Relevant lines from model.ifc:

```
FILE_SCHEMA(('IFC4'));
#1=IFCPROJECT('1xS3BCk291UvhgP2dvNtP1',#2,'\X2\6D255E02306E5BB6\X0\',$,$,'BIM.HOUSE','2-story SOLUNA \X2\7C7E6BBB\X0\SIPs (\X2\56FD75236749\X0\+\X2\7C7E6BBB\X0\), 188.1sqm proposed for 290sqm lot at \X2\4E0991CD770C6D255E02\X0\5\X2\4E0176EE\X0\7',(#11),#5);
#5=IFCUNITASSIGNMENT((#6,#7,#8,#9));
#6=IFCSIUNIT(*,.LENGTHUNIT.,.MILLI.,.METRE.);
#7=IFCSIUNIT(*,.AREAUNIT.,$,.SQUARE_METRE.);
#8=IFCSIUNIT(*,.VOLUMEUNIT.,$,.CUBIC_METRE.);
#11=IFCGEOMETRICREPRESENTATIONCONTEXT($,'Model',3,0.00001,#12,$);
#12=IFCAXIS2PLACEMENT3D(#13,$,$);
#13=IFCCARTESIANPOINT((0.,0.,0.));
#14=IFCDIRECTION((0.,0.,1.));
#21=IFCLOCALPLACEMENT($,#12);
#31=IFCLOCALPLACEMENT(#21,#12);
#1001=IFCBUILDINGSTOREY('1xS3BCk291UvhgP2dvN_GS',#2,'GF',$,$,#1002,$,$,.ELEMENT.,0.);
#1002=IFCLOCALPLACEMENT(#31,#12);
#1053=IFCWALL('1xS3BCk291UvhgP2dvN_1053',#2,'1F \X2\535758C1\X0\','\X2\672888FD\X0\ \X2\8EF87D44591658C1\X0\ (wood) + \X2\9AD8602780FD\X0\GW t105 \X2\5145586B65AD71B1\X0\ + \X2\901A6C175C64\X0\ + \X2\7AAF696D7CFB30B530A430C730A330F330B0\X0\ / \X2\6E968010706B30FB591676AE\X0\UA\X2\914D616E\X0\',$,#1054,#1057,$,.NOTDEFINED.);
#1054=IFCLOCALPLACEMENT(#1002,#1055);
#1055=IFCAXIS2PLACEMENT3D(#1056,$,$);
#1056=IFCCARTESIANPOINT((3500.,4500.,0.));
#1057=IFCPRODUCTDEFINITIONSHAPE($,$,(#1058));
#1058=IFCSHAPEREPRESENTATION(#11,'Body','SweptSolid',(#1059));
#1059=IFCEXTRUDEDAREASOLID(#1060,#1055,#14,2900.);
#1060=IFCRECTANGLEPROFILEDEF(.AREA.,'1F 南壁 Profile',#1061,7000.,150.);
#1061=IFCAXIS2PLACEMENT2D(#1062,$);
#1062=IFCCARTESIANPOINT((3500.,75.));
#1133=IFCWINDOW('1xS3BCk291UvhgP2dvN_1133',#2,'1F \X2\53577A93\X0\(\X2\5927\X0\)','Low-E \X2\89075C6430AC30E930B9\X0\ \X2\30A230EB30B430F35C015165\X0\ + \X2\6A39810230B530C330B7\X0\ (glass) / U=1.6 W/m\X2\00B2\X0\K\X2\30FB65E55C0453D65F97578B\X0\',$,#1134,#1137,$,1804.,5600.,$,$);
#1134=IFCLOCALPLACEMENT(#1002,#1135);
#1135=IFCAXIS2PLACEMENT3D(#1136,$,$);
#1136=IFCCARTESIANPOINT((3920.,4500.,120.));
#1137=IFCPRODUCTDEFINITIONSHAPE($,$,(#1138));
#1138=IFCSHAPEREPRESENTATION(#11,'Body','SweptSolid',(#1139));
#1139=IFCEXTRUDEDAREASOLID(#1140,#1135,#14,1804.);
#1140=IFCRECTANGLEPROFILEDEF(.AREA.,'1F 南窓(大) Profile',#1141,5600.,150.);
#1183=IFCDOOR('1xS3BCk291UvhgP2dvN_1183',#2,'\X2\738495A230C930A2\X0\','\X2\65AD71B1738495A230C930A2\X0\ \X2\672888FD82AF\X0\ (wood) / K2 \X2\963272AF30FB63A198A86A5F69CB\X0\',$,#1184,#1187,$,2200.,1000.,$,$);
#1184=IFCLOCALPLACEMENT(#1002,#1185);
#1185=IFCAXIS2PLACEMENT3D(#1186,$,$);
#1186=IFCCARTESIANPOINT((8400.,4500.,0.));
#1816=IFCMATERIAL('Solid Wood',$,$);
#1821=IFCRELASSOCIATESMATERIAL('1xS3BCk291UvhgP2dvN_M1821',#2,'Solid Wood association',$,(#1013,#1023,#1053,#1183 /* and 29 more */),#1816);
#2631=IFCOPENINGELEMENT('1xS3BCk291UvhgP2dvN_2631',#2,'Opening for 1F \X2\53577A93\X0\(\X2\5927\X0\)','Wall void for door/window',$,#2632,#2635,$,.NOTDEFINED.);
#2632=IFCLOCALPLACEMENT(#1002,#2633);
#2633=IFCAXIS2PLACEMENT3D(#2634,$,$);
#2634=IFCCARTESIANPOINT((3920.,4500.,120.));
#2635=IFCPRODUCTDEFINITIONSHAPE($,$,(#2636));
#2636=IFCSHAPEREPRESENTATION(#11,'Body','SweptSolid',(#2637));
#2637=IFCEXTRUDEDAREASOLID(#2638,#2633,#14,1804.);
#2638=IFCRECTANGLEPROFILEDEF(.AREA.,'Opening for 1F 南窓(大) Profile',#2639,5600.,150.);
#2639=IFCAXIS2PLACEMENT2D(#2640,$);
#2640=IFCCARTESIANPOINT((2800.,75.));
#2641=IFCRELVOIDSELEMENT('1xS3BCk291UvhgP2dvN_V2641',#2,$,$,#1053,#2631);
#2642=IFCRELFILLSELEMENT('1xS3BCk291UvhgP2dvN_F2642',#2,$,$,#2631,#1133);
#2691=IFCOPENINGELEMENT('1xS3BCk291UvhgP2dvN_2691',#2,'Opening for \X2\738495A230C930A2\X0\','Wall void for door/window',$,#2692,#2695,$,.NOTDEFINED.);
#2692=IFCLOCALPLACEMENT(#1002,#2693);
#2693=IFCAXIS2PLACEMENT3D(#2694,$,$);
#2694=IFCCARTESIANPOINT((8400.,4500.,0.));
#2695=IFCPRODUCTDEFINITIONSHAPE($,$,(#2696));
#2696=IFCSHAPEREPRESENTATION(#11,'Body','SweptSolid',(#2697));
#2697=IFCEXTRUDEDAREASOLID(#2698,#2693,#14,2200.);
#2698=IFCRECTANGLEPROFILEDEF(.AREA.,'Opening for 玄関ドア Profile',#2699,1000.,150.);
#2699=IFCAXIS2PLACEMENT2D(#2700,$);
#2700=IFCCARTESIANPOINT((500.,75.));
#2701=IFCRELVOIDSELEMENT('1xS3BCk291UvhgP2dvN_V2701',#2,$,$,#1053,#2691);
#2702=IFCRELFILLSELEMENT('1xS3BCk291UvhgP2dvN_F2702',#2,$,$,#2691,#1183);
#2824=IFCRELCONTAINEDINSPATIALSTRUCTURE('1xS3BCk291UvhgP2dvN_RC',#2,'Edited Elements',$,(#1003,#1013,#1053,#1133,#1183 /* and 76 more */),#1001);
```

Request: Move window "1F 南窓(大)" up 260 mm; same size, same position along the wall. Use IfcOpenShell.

```python
import numpy as np
import ifcopenshell
import ifcopenshell.api.geometry
import ifcopenshell.util.placement
import ifcopenshell.util.unit

model = ifcopenshell.open("model.ifc")
unit_scale = ifcopenshell.util.unit.calculate_unit_scale(model)

window = model.by_guid("1xS3BCk291UvhgP2dvN_1133")
opening = window.FillsVoids[0].RelatingOpeningElement
dz = 260.0

shift = np.array([0.0, 0.0, dz])
# The window is not placed relative to its opening, so move both.
for product in (opening, window):
    matrix = ifcopenshell.util.placement.get_local_placement(product.ObjectPlacement)
    matrix[:3, 3] += shift
    ifcopenshell.api.geometry.edit_object_placement(model, product=product, matrix=matrix, is_si=False)

print(f"moved by {dz * unit_scale:+.3f} m")

model.write("model_updated.ifc")
```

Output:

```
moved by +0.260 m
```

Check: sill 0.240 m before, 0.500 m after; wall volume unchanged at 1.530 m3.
